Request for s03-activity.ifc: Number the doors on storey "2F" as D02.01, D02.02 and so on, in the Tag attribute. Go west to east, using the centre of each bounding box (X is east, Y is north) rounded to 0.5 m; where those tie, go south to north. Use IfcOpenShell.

First a look at what the model holds.

```python
import ifcopenshell
import ifcopenshell.util.element
import ifcopenshell.util.placement

model = ifcopenshell.open("s03-activity.ifc")
print(model.schema)
storey = next(s for s in model.by_type("IfcBuildingStorey") if s.Name == "2F")
doors = [e for e in ifcopenshell.util.element.get_decomposition(storey) if e.is_a("IfcDoor")]
for e in sorted(doors, key=lambda e: e.id()):
    origin = ifcopenshell.util.placement.get_local_placement(e.ObjectPlacement)[:3, 3]
    print(e.id(), e.Tag, e.Name, origin.round(2) + 0.0, sep=" | ")
```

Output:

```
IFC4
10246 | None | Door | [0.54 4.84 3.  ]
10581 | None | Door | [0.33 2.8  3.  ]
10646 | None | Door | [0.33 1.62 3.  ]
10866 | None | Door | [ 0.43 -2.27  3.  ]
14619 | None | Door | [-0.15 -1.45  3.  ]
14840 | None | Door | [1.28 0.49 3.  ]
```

```python
import ifcopenshell
import ifcopenshell.geom
import ifcopenshell.util.element
import ifcopenshell.util.shape

model = ifcopenshell.open("s03-activity.ifc")
settings = ifcopenshell.geom.settings()
settings.set("use-world-coords", True)


def centre(element):
    shape = ifcopenshell.geom.create_shape(settings, element)
    return ifcopenshell.util.shape.get_bbox_centroid(shape.geometry)


storey = next(s for s in model.by_type("IfcBuildingStorey") if s.Name == "2F")
doors = [e for e in ifcopenshell.util.element.get_decomposition(storey) if e.is_a("IfcDoor")]

# Insertion points can sit at a corner or the storey origin, so sort by the geometry (in metres).
centres = {e: centre(e) for e in doors}
doors.sort(key=lambda e: (round(centres[e][0] / 0.5), centres[e][1]))

for i, e in enumerate(doors, start=1):
    number = f"D02.{i:02d}"
    e.Tag = number
    print(e.id(), number)

model.write("s03-activity_v2.ifc")
```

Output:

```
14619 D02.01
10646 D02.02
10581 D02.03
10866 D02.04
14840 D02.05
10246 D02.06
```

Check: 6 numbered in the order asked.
